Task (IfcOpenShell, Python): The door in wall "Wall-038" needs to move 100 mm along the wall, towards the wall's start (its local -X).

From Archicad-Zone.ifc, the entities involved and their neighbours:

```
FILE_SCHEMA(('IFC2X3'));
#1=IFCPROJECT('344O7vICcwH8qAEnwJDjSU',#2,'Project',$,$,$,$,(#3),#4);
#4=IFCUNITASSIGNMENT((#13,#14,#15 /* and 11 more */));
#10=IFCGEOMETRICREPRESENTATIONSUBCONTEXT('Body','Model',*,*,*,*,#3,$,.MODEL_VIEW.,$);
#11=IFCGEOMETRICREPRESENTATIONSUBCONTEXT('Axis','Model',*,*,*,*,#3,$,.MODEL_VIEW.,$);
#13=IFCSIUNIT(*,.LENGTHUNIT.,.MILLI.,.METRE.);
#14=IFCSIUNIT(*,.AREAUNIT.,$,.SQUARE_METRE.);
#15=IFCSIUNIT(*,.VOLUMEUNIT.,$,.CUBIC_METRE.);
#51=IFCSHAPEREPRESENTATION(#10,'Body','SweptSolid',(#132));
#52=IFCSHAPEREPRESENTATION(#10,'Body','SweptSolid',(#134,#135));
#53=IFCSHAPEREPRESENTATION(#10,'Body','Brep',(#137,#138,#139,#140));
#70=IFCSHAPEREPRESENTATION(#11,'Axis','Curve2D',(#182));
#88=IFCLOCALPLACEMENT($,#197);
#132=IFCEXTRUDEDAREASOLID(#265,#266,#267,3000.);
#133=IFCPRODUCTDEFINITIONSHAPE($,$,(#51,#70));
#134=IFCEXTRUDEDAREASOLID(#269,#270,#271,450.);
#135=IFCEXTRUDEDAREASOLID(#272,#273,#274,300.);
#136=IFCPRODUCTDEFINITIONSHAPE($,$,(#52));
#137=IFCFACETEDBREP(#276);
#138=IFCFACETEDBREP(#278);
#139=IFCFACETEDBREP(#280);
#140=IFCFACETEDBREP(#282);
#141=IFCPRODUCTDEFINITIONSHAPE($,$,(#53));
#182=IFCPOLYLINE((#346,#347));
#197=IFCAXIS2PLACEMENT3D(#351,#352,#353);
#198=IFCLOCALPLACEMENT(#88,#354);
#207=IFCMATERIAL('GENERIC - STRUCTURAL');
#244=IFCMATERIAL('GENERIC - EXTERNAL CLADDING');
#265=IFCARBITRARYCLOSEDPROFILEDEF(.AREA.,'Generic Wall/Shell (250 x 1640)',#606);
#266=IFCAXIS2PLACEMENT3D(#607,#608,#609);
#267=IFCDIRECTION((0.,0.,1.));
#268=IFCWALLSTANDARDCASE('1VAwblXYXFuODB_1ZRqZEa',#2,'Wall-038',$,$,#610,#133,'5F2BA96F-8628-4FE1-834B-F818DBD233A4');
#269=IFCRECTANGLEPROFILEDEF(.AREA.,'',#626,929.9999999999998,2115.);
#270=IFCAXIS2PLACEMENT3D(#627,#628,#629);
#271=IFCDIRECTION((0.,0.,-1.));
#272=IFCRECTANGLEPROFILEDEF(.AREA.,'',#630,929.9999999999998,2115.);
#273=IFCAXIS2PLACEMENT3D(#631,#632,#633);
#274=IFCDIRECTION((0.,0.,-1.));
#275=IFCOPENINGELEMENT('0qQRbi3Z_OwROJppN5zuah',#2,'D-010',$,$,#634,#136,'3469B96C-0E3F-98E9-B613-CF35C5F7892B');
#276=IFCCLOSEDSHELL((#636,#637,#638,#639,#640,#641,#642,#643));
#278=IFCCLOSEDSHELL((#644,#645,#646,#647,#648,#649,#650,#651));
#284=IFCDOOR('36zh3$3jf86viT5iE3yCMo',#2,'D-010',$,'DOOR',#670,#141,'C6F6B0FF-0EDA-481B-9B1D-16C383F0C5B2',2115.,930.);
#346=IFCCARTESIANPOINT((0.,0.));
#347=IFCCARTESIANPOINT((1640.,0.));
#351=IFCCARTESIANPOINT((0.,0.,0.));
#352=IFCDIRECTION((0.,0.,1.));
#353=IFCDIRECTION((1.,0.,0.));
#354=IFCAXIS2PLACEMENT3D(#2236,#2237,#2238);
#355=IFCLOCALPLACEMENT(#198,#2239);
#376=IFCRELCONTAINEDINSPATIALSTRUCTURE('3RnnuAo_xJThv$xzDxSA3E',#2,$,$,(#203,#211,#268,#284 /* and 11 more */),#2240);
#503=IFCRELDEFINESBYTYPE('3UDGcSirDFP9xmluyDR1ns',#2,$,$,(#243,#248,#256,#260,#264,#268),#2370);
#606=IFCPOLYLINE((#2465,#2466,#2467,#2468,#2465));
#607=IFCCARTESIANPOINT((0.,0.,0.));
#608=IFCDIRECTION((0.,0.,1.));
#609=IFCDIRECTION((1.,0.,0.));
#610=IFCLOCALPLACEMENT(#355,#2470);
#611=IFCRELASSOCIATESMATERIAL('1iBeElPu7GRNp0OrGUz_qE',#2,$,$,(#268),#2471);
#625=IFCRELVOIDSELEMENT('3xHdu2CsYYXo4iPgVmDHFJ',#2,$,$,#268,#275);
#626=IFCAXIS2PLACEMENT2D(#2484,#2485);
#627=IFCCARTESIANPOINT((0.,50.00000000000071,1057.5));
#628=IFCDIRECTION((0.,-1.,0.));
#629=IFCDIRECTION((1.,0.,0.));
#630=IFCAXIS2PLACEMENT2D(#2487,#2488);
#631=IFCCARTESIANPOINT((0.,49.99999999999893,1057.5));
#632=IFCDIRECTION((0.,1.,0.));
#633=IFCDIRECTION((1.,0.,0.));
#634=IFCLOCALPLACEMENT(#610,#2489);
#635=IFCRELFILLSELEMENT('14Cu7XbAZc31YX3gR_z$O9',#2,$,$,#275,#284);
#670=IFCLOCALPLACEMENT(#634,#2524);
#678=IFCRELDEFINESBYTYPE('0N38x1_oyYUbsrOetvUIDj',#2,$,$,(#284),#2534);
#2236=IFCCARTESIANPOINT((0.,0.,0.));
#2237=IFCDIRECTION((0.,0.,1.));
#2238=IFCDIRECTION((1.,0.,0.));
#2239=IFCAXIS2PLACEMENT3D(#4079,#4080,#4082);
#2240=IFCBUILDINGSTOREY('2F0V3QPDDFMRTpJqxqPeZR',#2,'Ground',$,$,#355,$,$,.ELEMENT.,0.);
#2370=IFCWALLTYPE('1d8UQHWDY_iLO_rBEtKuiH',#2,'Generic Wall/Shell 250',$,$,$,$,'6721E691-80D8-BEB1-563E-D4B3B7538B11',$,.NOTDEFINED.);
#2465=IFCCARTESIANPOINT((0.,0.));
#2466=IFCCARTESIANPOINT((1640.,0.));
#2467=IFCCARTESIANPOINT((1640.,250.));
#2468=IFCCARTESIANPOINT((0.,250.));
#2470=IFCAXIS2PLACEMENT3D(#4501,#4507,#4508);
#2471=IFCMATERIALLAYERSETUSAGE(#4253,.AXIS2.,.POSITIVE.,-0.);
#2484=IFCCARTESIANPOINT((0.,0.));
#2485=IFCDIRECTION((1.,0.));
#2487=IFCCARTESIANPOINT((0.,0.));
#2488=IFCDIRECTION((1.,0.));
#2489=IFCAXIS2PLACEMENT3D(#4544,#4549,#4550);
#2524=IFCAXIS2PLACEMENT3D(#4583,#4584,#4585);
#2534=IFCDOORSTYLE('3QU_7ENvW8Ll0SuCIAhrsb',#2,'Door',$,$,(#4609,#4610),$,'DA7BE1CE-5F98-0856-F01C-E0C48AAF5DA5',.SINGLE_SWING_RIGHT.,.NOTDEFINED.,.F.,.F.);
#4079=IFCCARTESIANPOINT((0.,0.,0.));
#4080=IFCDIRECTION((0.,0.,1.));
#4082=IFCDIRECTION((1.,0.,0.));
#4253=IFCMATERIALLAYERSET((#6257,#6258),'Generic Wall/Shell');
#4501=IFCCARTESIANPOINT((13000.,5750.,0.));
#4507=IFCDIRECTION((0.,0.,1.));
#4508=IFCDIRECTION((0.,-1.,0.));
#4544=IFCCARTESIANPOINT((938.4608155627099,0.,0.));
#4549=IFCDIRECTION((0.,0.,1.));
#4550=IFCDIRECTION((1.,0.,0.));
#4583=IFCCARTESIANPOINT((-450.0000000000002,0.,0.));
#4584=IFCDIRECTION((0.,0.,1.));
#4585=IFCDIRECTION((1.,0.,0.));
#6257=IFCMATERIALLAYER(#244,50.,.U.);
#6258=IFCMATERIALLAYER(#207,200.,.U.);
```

```python
import ifcopenshell
import ifcopenshell.api.geometry
import ifcopenshell.util.placement
import ifcopenshell.util.unit

model = ifcopenshell.open("Archicad-Zone.ifc")
unit_scale = ifcopenshell.util.unit.calculate_unit_scale(model)

door = model.by_guid("36zh3$3jf86viT5iE3yCMo")
opening = door.FillsVoids[0].RelatingOpeningElement
wall = opening.VoidsElements[0].RelatingBuildingElement

wall_matrix = ifcopenshell.util.placement.get_local_placement(wall.ObjectPlacement)
shift = wall_matrix[:3, 0] * -0.1 / unit_scale
before = ifcopenshell.util.placement.get_local_placement(door.ObjectPlacement)[:3, 3].copy()

# The door is placed relative to its opening, so it follows when the opening moves.
matrix = ifcopenshell.util.placement.get_local_placement(opening.ObjectPlacement)
matrix[:3, 3] += shift
ifcopenshell.api.geometry.edit_object_placement(
    model, product=opening, matrix=matrix, is_si=False, should_transform_children=True
)

after = ifcopenshell.util.placement.get_local_placement(door.ObjectPlacement)[:3, 3]
print("door moved by", (after - before).round(3) + 0.0)

model.write("Archicad-Zone_rev.ifc")
```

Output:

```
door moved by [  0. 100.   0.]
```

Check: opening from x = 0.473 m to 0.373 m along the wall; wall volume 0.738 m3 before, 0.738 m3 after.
